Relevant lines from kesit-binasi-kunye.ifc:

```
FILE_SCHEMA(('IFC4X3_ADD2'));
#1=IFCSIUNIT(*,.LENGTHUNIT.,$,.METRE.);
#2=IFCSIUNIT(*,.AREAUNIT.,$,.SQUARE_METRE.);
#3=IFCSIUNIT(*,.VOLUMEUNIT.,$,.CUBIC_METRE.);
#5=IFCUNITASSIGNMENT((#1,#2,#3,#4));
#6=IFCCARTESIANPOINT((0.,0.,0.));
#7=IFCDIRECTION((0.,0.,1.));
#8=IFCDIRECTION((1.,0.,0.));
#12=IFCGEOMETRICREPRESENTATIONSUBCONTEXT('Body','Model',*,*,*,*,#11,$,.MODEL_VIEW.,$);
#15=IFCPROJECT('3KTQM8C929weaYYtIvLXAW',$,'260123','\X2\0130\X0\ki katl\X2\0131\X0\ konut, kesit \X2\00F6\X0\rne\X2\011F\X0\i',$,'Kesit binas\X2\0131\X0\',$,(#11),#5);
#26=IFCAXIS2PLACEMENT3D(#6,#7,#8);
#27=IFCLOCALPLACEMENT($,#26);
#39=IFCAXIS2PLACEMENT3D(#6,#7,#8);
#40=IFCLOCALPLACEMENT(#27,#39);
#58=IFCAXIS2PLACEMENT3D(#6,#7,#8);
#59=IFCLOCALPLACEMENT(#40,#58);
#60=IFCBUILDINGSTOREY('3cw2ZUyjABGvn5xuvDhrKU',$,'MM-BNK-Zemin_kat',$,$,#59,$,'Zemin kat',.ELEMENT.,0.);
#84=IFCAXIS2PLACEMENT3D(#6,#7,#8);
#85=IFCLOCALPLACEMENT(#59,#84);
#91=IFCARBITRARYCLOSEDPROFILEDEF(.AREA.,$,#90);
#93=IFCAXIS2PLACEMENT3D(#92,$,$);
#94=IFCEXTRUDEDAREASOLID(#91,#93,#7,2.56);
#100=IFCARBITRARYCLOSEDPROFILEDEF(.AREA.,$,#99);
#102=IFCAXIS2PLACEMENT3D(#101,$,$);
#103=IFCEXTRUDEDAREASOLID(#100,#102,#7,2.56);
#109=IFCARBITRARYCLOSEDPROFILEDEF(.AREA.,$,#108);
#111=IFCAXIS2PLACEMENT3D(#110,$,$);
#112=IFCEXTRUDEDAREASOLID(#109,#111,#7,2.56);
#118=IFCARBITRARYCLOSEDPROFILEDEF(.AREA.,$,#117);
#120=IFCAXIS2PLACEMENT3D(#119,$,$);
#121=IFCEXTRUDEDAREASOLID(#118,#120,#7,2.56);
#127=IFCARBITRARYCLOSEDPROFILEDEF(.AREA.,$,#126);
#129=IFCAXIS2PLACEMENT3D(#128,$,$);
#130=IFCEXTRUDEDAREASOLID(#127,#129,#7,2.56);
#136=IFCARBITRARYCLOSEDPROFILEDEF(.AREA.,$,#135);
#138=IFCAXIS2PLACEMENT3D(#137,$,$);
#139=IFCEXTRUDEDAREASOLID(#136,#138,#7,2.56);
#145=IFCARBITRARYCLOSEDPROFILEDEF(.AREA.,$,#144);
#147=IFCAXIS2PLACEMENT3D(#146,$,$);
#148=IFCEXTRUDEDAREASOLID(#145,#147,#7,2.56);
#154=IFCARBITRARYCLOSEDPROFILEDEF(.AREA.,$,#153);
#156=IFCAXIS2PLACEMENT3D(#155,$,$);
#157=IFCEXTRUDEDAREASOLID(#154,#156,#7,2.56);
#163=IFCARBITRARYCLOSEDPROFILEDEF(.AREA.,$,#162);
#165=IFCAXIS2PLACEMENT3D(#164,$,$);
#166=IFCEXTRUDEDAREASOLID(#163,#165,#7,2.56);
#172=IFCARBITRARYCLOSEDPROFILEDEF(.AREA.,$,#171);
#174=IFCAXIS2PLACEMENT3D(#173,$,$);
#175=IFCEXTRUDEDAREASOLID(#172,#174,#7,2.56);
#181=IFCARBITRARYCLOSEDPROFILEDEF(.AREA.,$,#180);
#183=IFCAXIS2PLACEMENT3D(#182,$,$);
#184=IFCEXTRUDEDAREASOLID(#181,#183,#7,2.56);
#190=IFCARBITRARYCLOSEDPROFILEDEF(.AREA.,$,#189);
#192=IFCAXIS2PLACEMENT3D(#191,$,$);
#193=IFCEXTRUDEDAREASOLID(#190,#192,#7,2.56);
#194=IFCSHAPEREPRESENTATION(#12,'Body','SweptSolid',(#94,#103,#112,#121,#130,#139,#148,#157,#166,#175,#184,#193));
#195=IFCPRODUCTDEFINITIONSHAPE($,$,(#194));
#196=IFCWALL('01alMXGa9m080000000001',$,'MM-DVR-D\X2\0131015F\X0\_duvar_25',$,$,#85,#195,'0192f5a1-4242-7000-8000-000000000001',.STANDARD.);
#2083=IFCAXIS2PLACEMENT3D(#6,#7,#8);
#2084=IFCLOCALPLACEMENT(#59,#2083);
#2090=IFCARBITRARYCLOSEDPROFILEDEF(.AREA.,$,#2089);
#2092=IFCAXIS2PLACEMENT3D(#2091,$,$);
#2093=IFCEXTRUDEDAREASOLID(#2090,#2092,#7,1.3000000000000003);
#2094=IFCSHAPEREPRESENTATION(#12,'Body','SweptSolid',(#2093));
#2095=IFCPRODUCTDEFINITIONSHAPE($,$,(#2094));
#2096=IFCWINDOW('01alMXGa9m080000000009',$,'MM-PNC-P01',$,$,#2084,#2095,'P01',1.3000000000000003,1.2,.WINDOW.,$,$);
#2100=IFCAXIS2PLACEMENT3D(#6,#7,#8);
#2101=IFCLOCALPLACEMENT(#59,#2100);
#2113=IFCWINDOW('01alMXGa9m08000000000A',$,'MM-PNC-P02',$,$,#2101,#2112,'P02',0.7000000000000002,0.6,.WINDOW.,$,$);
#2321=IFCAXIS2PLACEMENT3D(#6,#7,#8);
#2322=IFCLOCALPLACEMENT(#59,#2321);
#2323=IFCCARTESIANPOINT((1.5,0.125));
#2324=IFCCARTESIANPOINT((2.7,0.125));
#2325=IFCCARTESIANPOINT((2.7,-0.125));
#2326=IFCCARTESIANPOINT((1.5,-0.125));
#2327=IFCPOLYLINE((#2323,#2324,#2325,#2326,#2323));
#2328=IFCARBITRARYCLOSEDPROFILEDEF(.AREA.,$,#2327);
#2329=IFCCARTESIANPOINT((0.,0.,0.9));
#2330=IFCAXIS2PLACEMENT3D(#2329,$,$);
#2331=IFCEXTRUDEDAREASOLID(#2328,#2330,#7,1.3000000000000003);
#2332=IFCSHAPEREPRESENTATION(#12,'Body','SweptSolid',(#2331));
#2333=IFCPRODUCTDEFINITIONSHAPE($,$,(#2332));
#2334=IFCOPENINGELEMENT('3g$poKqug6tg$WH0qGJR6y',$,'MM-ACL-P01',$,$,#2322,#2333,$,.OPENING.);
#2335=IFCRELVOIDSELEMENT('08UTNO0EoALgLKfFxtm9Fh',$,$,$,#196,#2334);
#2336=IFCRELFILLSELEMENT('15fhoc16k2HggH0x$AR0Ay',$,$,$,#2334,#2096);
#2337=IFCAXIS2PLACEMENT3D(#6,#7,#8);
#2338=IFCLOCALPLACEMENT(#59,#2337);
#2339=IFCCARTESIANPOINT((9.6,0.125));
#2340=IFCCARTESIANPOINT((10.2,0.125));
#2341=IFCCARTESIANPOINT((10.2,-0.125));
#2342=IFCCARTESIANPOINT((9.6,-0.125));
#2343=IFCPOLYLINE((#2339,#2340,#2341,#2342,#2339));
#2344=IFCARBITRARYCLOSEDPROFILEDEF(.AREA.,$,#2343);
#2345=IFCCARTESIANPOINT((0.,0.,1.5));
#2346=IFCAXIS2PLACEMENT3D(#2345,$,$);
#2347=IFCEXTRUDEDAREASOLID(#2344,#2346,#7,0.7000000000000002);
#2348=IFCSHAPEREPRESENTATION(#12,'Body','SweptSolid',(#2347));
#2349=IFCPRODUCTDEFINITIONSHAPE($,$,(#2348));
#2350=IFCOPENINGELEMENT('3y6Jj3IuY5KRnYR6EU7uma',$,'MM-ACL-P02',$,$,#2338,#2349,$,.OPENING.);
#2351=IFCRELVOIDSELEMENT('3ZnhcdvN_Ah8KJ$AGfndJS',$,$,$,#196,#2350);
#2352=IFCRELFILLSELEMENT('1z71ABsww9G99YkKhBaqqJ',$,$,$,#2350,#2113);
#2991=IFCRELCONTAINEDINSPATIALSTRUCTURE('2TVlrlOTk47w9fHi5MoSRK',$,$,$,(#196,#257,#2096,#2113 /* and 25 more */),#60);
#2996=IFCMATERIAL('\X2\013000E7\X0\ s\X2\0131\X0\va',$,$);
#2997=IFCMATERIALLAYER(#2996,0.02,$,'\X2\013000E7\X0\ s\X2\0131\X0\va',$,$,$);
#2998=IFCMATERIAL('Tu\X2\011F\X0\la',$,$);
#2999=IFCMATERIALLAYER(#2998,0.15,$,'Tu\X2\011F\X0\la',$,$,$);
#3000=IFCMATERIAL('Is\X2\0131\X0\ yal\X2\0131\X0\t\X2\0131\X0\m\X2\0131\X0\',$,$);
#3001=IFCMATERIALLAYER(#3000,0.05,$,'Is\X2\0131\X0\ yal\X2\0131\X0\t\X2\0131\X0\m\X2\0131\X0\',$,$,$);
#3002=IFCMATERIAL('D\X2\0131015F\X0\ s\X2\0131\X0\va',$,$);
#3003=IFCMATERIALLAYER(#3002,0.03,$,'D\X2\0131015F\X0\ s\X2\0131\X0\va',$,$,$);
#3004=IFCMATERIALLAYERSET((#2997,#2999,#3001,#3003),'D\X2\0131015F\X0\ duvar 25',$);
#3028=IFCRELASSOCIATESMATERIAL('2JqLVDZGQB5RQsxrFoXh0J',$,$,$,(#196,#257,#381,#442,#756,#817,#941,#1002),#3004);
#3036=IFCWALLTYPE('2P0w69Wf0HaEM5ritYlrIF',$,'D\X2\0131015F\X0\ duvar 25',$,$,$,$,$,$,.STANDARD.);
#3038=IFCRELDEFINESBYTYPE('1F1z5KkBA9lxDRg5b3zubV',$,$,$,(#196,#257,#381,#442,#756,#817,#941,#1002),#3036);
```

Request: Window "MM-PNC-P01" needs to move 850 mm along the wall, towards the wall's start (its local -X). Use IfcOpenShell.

```python
import ifcopenshell
import ifcopenshell.api.geometry
import ifcopenshell.util.placement
import ifcopenshell.util.unit

model = ifcopenshell.open("kesit-binasi-kunye.ifc")
unit_scale = ifcopenshell.util.unit.calculate_unit_scale(model)

window = model.by_guid("01alMXGa9m080000000009")
opening = window.FillsVoids[0].RelatingOpeningElement
wall = opening.VoidsElements[0].RelatingBuildingElement

wall_matrix = ifcopenshell.util.placement.get_local_placement(wall.ObjectPlacement)
shift = wall_matrix[:3, 0] * -0.85 / unit_scale
before = ifcopenshell.util.placement.get_local_placement(window.ObjectPlacement)[:3, 3].copy()

# The window is not placed relative to its opening, so move both.
for product in (opening, window):
    matrix = ifcopenshell.util.placement.get_local_placement(product.ObjectPlacement)
    matrix[:3, 3] += shift
    ifcopenshell.api.geometry.edit_object_placement(model, product=product, matrix=matrix, is_si=False)

after = ifcopenshell.util.placement.get_local_placement(window.ObjectPlacement)[:3, 3]
print("window moved by", (after - before).round(3) + 0.0)

model.write("kesit-binasi-kunye_edited.ifc")
```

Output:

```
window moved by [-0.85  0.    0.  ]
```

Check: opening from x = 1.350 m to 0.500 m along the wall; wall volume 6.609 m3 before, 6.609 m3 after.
